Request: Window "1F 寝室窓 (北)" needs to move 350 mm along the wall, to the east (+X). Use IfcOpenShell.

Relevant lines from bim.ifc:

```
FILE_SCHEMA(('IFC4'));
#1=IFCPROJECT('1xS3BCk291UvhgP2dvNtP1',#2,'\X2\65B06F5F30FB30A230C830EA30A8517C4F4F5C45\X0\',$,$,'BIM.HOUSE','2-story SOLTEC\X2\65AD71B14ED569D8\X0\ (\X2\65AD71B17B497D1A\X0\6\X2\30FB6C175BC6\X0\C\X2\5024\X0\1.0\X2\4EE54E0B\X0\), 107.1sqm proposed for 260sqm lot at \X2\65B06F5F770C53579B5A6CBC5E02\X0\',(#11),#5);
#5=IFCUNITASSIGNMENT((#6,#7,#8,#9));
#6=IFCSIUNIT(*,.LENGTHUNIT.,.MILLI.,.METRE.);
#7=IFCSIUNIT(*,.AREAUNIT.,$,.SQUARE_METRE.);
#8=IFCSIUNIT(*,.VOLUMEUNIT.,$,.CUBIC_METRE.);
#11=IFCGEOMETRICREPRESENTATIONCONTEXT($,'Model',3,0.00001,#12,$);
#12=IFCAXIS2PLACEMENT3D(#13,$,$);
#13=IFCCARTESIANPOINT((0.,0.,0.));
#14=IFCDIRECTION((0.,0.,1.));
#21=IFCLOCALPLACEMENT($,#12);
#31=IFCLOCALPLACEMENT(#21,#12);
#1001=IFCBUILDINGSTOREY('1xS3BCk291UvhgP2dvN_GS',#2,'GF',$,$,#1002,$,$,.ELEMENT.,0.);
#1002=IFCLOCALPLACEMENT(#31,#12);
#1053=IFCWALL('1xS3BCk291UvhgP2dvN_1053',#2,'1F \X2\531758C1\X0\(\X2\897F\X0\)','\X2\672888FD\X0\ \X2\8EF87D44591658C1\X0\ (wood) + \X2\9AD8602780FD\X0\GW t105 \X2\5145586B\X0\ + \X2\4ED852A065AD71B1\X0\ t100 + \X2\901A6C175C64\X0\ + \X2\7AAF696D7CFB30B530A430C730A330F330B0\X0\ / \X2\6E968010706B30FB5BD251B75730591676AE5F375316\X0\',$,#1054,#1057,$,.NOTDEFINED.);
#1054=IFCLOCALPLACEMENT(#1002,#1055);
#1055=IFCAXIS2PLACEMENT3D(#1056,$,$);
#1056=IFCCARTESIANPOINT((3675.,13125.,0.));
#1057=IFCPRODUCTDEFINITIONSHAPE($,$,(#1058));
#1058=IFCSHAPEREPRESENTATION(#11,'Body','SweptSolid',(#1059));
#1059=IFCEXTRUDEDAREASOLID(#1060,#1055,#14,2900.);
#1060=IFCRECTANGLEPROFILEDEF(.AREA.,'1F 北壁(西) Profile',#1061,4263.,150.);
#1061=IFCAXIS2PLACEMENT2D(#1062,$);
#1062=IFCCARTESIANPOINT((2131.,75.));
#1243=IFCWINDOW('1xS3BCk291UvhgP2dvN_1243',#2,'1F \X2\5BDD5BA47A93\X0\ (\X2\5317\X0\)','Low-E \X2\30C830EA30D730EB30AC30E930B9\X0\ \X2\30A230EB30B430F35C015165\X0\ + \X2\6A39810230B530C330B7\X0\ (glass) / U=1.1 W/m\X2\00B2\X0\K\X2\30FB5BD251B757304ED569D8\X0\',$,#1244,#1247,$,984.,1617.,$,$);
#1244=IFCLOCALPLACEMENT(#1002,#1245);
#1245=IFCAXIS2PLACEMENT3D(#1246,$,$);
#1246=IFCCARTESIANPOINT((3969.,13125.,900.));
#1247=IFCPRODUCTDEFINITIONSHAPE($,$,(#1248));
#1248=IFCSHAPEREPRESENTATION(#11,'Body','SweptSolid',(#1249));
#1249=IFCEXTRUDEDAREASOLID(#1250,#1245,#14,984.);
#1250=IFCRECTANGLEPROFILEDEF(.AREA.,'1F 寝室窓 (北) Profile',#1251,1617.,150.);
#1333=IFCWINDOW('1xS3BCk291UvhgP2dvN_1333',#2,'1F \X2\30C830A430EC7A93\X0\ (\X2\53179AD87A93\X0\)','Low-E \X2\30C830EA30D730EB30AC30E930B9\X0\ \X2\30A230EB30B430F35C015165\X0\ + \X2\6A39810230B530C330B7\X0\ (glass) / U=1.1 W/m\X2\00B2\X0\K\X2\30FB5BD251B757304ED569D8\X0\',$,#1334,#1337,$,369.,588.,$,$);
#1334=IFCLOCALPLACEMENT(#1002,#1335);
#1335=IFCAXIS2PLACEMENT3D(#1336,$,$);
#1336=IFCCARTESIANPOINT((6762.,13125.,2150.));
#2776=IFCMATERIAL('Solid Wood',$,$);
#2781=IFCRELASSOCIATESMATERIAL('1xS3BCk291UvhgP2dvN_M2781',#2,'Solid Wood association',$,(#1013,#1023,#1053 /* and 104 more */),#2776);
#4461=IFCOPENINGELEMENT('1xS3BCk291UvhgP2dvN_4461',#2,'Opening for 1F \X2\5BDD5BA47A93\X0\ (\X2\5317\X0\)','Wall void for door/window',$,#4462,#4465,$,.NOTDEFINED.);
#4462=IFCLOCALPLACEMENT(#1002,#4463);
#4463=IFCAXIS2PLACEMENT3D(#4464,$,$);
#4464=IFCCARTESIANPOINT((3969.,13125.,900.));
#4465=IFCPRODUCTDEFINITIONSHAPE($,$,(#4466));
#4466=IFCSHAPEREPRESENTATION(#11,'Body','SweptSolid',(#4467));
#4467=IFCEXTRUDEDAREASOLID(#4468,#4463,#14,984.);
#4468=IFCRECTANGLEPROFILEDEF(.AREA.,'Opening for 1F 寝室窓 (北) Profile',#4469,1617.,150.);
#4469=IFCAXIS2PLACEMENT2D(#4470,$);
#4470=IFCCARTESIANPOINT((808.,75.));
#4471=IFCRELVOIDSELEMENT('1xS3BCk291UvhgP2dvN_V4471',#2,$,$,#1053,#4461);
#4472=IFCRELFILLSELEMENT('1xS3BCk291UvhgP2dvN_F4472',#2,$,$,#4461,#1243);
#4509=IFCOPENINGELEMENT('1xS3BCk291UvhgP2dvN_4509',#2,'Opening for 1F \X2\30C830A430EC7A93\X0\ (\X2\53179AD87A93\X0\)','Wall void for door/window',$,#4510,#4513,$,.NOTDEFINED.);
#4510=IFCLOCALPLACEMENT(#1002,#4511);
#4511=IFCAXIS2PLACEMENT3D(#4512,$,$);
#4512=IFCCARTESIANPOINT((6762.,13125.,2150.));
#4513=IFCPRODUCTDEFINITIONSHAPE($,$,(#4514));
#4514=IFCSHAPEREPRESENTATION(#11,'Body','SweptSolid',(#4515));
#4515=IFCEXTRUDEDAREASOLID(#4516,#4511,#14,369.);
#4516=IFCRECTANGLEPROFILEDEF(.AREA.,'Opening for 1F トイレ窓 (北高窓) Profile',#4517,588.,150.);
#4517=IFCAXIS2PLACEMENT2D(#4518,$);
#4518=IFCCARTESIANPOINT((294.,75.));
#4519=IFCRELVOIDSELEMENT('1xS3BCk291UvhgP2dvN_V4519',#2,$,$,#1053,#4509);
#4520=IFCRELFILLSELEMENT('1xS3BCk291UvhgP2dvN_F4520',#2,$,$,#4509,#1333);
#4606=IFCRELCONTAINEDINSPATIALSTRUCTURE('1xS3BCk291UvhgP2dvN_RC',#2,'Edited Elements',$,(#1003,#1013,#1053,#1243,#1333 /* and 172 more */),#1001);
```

```python
import ifcopenshell
import ifcopenshell.api.geometry
import ifcopenshell.util.placement
import ifcopenshell.util.unit

model = ifcopenshell.open("bim.ifc")
unit_scale = ifcopenshell.util.unit.calculate_unit_scale(model)

window = model.by_guid("1xS3BCk291UvhgP2dvN_1243")
opening = window.FillsVoids[0].RelatingOpeningElement
wall = opening.VoidsElements[0].RelatingBuildingElement

wall_matrix = ifcopenshell.util.placement.get_local_placement(wall.ObjectPlacement)
shift = wall_matrix[:3, 0] * 0.35 / unit_scale
before = ifcopenshell.util.placement.get_local_placement(window.ObjectPlacement)[:3, 3].copy()

# The window is not placed relative to its opening, so move both.
for product in (opening, window):
    matrix = ifcopenshell.util.placement.get_local_placement(product.ObjectPlacement)
    matrix[:3, 3] += shift
    ifcopenshell.api.geometry.edit_object_placement(model, product=product, matrix=matrix, is_si=False)

after = ifcopenshell.util.placement.get_local_placement(window.ObjectPlacement)[:3, 3]
print("window moved by", (after - before).round(3) + 0.0)

model.write("bim_updated.ifc")
```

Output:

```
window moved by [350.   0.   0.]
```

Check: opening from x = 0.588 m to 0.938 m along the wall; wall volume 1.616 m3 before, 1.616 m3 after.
